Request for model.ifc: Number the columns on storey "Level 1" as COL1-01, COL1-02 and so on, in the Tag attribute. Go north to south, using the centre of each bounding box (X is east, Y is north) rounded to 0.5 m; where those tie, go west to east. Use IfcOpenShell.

First a look at what the model holds.

```python
import ifcopenshell
import ifcopenshell.util.element
import ifcopenshell.util.placement

model = ifcopenshell.open("model.ifc")
print(model.schema)
storey = next(s for s in model.by_type("IfcBuildingStorey") if s.Name == "Level 1")
columns = [e for e in ifcopenshell.util.element.get_decomposition(storey) if e.is_a("IfcColumn")]
for e in sorted(columns, key=lambda e: e.id()):
    origin = ifcopenshell.util.placement.get_local_placement(e.ObjectPlacement)[:3, 3]
    print(e.id(), e.Tag, e.Name, origin.round(2) + 0.0, sep=" | ")
```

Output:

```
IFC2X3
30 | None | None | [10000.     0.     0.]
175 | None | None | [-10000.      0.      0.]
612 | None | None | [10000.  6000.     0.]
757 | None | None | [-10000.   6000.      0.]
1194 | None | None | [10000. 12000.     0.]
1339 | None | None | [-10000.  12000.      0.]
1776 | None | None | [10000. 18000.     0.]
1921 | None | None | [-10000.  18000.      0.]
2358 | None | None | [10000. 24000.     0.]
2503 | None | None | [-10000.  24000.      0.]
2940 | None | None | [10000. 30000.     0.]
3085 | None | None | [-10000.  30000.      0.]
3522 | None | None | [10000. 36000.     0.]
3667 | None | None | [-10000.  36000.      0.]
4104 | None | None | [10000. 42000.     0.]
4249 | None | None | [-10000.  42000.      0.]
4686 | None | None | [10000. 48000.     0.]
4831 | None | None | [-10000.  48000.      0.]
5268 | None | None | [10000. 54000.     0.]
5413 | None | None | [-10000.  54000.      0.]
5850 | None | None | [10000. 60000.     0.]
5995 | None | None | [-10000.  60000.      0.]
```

```python
import ifcopenshell
import ifcopenshell.geom
import ifcopenshell.util.element
import ifcopenshell.util.shape

model = ifcopenshell.open("model.ifc")
settings = ifcopenshell.geom.settings()
settings.set("use-world-coords", True)


def centre(element):
    shape = ifcopenshell.geom.create_shape(settings, element)
    return ifcopenshell.util.shape.get_bbox_centroid(shape.geometry)


storey = next(s for s in model.by_type("IfcBuildingStorey") if s.Name == "Level 1")
columns = [e for e in ifcopenshell.util.element.get_decomposition(storey) if e.is_a("IfcColumn")]

# Insertion points can sit at a corner or the storey origin, so sort by the geometry (in metres).
centres = {e: centre(e) for e in columns}
columns.sort(key=lambda e: (-round(centres[e][1] / 0.5), centres[e][0]))

for i, e in enumerate(columns, start=1):
    number = f"COL1-{i:02d}"
    e.Tag = number
    print(e.id(), number)

model.write("model_rev.ifc")
```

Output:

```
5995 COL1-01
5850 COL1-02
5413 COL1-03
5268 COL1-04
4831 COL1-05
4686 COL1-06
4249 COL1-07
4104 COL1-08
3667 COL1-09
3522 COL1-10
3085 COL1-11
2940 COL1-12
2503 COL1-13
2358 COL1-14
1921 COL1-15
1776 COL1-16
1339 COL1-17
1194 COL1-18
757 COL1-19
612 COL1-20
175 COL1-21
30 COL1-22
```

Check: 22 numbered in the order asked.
